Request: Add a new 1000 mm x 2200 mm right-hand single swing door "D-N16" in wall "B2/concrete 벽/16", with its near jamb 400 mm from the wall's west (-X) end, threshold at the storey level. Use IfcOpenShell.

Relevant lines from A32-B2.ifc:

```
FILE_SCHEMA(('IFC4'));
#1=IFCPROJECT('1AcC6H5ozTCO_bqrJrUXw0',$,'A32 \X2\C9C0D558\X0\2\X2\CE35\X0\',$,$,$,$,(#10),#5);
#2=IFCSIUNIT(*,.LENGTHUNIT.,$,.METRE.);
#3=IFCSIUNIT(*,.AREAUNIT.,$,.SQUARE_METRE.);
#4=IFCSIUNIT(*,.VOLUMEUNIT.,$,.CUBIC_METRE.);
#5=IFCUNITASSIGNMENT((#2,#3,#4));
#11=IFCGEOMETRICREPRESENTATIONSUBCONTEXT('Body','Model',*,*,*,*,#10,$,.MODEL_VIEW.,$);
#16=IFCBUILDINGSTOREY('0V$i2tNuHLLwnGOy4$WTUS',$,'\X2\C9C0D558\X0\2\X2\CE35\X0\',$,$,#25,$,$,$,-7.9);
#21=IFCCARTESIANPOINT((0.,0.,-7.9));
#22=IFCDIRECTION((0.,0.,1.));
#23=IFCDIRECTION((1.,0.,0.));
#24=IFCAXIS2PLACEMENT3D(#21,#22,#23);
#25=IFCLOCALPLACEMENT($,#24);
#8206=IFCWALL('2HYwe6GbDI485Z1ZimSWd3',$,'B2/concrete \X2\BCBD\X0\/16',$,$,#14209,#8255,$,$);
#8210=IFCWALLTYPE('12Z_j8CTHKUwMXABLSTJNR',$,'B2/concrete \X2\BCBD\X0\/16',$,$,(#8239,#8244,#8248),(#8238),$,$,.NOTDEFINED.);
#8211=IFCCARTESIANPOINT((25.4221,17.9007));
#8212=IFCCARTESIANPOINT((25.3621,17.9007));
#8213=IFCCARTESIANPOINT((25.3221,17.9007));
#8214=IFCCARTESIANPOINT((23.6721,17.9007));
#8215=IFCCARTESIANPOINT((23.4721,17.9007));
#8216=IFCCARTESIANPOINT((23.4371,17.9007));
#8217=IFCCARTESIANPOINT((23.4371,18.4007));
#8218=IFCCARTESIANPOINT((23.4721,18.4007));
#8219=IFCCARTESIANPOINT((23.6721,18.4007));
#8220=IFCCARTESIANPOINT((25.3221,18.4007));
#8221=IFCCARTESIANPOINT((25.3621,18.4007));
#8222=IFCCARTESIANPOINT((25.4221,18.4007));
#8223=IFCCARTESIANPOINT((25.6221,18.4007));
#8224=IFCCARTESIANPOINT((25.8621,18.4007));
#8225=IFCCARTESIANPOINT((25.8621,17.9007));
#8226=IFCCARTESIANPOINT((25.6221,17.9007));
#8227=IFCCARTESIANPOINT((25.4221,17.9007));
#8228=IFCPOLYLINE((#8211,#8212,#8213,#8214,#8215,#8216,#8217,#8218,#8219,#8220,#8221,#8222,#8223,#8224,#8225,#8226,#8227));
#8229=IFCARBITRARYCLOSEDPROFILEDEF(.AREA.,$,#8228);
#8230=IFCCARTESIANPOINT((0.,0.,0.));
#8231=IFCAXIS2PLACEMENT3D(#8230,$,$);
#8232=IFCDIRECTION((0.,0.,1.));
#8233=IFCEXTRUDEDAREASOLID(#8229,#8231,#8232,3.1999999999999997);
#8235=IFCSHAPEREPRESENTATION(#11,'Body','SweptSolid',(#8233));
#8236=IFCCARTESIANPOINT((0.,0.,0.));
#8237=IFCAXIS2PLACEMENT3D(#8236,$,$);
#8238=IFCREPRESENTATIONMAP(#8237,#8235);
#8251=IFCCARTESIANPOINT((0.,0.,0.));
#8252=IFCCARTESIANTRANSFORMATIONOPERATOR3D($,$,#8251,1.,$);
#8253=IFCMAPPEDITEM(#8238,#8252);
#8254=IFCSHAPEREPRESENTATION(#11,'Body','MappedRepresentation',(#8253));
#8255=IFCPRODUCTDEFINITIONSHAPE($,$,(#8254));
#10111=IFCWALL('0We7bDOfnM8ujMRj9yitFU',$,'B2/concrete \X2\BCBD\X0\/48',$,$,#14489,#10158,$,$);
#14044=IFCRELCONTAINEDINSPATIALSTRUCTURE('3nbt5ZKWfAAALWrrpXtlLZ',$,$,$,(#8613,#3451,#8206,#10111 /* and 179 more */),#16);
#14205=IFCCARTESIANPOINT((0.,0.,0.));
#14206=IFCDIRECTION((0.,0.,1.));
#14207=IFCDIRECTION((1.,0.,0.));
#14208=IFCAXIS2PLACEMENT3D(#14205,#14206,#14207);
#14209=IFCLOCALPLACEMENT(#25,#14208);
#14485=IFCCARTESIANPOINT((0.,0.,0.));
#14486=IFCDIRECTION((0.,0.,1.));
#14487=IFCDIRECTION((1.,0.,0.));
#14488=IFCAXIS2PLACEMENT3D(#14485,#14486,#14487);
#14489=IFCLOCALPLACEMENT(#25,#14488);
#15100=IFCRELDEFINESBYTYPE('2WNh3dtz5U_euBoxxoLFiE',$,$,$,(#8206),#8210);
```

```python
import numpy as np
import ifcopenshell
import ifcopenshell.api.feature
import ifcopenshell.api.geometry
import ifcopenshell.api.root
import ifcopenshell.api.spatial
import ifcopenshell.geom
import ifcopenshell.util.element
import ifcopenshell.util.placement
import ifcopenshell.util.representation
import ifcopenshell.util.shape
import ifcopenshell.util.unit

model = ifcopenshell.open("A32-B2.ifc")
unit_scale = ifcopenshell.util.unit.calculate_unit_scale(model)
settings = ifcopenshell.geom.settings()


def volume(element):
    """Net volume in cubic metres, openings subtracted."""
    shape = ifcopenshell.geom.create_shape(settings, element)
    return ifcopenshell.util.shape.get_volume(shape.geometry)


wall = model.by_id(8206)
storey = ifcopenshell.util.element.get_container(wall, ifc_class="IfcBuildingStorey")
context = ifcopenshell.util.representation.get_context(model, "Model", "Body", "MODEL_VIEW")
before = volume(wall)

width, height, from_end, sill = 1, 2.2, 0.4, 0.0  # metres

# The wall runs along its own X axis, and the end named is its -X end.
wall_shape = ifcopenshell.geom.create_shape(settings, wall)
x, y, z = ifcopenshell.util.shape.get_vertices(wall_shape.geometry).T
start = x.min() + from_end
face, thickness = float(y.min()), float(y.max() - y.min())
wall_matrix = ifcopenshell.util.placement.get_local_placement(wall.ObjectPlacement)
level = ifcopenshell.util.placement.get_local_placement(storey.ObjectPlacement)[2, 3]


def in_wall(x, y):
    """Placement at x, y metres in the wall's axes, at sill height."""
    matrix = wall_matrix.copy()
    matrix[:, 3] = wall_matrix @ np.array([x / unit_scale, y / unit_scale, 0.0, 1.0])
    matrix[2, 3] = level + sill / unit_scale
    return matrix


# Opening: a box that overshoots both wall faces by 50 mm.
opening = ifcopenshell.api.root.create_entity(model, ifc_class="IfcOpeningElement", predefined_type="OPENING")
box = ifcopenshell.api.geometry.add_wall_representation(
    model, context=context, length=width, height=height, thickness=thickness + 0.1
)
ifcopenshell.api.geometry.assign_representation(model, product=opening, representation=box)
ifcopenshell.api.geometry.edit_object_placement(model, product=opening, matrix=in_wall(start, face - 0.05), is_si=False)
ifcopenshell.api.feature.add_feature(model, feature=opening, element=wall)

door = ifcopenshell.api.root.create_entity(model, ifc_class="IfcDoor", name="D-N16", predefined_type="DOOR")
door.OverallWidth, door.OverallHeight = width / unit_scale, height / unit_scale
door.OperationType = "SINGLE_SWING_RIGHT"
body = ifcopenshell.api.geometry.add_door_representation(
    model,
    context=context,
    overall_width=door.OverallWidth,
    overall_height=door.OverallHeight,
    operation_type="SINGLE_SWING_RIGHT",
    lining_properties={"LiningDepth": thickness / unit_scale, "ThresholdDepth": thickness / unit_scale},
)
ifcopenshell.api.geometry.assign_representation(model, product=door, representation=body)
ifcopenshell.api.spatial.assign_container(model, products=[door], relating_structure=storey)
ifcopenshell.api.feature.add_filling(model, opening=opening, element=door)

# The lining spans the wall, so the door starts at the wall face.
ifcopenshell.api.geometry.edit_object_placement(model, product=door, matrix=in_wall(start, face), is_si=False)

after = volume(wall)

print(f"wall volume {before:.3f} -> {after:.3f} m3")

model.write("A32-B2_v2.ifc")
```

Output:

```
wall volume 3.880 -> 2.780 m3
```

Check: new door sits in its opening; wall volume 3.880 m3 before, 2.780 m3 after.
